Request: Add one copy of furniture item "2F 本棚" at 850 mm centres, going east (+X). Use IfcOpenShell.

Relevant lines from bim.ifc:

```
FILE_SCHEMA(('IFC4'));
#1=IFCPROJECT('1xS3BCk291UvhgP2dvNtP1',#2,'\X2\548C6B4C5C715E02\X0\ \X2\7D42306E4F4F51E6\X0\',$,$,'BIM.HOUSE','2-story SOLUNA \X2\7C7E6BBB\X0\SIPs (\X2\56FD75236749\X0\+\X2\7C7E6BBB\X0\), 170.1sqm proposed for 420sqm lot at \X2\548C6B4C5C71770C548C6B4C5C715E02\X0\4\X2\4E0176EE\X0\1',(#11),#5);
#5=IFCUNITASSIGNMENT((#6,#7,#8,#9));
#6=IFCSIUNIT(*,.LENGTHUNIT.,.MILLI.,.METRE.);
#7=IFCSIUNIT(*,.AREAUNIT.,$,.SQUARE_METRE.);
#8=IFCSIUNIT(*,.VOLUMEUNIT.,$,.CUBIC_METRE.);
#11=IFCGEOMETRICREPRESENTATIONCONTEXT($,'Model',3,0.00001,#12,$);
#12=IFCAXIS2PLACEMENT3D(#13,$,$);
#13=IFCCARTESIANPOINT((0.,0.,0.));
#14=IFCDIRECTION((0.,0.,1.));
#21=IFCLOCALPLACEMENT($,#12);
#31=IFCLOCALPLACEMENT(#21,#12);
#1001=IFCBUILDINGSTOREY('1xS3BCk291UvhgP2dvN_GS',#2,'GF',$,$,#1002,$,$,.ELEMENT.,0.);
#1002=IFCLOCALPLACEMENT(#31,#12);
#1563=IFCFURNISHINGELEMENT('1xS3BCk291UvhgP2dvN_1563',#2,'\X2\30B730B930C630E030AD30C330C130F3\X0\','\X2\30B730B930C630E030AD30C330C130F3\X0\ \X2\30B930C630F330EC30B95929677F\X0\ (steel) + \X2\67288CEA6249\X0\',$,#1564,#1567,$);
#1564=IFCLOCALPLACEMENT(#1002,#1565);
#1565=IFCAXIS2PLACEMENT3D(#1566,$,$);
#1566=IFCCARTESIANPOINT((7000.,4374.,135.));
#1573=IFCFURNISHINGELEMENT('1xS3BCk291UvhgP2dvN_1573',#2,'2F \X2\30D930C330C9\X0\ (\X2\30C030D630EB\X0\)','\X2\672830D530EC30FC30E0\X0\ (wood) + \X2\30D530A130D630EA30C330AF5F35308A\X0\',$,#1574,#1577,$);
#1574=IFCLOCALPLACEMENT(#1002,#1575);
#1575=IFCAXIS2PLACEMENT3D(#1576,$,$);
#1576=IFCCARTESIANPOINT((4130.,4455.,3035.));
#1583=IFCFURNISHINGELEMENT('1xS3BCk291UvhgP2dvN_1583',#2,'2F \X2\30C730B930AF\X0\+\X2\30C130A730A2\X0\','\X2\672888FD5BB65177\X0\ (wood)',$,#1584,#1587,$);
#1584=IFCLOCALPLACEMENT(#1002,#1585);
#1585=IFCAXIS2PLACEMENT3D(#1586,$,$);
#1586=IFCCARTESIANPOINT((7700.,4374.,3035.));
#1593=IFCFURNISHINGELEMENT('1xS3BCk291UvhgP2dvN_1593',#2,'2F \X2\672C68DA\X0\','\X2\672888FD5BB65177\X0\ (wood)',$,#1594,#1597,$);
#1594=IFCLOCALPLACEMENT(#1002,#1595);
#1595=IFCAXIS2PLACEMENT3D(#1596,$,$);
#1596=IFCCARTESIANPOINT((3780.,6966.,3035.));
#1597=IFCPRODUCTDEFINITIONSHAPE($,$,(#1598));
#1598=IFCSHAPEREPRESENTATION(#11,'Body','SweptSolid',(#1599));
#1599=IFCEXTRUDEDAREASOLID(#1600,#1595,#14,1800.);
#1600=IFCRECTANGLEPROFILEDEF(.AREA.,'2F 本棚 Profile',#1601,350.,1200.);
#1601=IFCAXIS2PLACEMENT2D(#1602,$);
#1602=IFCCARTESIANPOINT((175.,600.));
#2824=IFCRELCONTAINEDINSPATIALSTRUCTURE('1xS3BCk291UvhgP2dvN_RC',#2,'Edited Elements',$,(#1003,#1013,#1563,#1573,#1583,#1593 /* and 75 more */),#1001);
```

```python
import numpy as np
import ifcopenshell
import ifcopenshell.api.geometry
import ifcopenshell.api.root
import ifcopenshell.util.element
import ifcopenshell.util.placement
import ifcopenshell.util.unit

model = ifcopenshell.open("bim.ifc")
unit_scale = ifcopenshell.util.unit.calculate_unit_scale(model)


def reuse_history(source, copy):
    """copy_class also copies each property set's owner history, people and application; keep the originals."""
    for rel in copy.IsDefinedBy:
        if rel.is_a("IfcRelDefinesByProperties") and (history := rel.RelatingPropertyDefinition.OwnerHistory):
            rel.RelatingPropertyDefinition.OwnerHistory = source.OwnerHistory
            ifcopenshell.util.element.remove_deep2(model, history)


source = model.by_guid("1xS3BCk291UvhgP2dvN_1593")
base = ifcopenshell.util.placement.get_local_placement(source.ObjectPlacement)
step = np.array([1.0, 0.0, 0.0]) * 0.85 / unit_scale

for i in range(1, 2):
    copy = ifcopenshell.api.root.copy_class(model, product=source)
    copy.Representation = ifcopenshell.util.element.copy_deep(
        model, source.Representation, exclude=["IfcGeometricRepresentationContext", "IfcRepresentationMap"]
    )
    reuse_history(source, copy)
    matrix = base.copy()
    matrix[:3, 3] += i * step
    print("added at", matrix[:3, 3].round(3) + 0.0)
    ifcopenshell.api.geometry.edit_object_placement(model, product=copy, matrix=matrix, is_si=False)

model.write("bim_v2.ifc")
```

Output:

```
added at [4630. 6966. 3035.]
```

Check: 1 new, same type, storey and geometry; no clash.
